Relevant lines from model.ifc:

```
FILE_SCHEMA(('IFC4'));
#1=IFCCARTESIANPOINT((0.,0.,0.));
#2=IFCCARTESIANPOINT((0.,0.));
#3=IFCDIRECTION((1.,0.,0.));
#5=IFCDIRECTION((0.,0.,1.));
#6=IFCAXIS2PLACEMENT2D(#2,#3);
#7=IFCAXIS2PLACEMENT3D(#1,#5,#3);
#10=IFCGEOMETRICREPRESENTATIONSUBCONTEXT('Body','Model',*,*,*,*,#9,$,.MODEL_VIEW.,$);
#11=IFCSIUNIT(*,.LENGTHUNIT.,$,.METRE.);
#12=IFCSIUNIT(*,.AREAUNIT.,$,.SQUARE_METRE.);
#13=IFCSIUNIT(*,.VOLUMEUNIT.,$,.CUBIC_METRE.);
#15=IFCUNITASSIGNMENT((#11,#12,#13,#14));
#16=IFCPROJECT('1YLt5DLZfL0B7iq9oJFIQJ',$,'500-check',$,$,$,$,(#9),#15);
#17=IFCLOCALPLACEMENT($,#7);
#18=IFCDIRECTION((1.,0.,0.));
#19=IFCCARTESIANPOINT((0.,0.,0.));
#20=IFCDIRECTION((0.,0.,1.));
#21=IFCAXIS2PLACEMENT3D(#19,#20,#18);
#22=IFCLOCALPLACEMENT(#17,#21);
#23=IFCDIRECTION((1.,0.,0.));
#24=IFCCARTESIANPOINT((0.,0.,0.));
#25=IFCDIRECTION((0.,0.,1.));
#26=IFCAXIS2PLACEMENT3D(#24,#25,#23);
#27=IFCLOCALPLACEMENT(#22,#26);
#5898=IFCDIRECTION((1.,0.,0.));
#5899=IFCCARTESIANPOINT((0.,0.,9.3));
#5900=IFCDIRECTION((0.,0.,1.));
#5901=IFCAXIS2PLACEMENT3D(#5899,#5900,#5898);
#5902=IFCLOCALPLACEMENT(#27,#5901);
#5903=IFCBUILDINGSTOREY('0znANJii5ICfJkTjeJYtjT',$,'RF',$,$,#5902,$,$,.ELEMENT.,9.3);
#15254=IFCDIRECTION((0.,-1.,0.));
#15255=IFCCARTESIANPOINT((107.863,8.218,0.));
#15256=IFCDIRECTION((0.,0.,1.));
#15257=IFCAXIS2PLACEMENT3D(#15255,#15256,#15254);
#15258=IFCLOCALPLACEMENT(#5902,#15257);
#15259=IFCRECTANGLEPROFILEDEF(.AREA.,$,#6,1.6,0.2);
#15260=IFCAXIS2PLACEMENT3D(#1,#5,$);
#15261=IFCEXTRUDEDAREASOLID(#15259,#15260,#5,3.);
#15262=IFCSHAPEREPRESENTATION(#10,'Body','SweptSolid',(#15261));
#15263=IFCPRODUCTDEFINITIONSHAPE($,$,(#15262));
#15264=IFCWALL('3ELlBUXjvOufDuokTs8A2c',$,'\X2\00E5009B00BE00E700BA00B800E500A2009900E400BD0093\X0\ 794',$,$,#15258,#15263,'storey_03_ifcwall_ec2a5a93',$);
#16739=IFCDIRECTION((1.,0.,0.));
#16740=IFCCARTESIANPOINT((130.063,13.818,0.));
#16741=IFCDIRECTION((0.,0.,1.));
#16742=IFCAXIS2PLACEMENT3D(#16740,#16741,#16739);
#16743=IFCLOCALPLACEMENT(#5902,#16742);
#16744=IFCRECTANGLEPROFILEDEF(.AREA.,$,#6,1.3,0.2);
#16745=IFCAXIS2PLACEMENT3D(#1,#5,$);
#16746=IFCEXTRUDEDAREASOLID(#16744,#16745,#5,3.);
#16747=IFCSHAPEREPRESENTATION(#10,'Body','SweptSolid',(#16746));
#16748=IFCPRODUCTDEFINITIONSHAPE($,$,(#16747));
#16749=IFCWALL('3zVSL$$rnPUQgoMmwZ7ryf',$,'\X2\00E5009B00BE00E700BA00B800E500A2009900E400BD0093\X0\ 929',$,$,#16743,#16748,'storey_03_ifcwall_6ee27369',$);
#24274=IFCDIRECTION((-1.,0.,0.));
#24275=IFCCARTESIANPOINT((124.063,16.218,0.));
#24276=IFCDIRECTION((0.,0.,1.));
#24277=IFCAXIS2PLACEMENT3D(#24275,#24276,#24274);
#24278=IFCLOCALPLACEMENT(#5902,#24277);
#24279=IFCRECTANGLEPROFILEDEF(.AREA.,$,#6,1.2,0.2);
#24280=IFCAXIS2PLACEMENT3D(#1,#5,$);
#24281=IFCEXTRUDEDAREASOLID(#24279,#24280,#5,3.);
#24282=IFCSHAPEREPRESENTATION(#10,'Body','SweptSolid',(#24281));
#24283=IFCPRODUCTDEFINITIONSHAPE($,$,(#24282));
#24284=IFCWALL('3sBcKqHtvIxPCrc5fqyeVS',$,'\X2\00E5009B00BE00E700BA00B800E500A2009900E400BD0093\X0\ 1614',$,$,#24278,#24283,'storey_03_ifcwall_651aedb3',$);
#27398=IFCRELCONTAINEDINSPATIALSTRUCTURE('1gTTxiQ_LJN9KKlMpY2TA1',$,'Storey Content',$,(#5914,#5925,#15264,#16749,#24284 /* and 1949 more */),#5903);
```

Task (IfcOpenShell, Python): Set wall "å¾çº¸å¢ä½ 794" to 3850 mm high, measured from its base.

```python
import ifcopenshell
import ifcopenshell.geom
import ifcopenshell.util.representation
import ifcopenshell.util.shape
import ifcopenshell.util.unit

model = ifcopenshell.open("model.ifc")
unit_scale = ifcopenshell.util.unit.calculate_unit_scale(model)
settings = ifcopenshell.geom.settings()


def volume(element):
    """Net volume in cubic metres, openings subtracted."""
    shape = ifcopenshell.geom.create_shape(settings, element)
    return ifcopenshell.util.shape.get_volume(shape.geometry)


wall = model.by_id(15264)
before = volume(wall)

body = ifcopenshell.util.representation.get_representation(wall, "Model", "Body")
solid = body.Items[0]
old_height = solid.Depth
solid.Depth = 3.85 / unit_scale
after = volume(wall)

print(f"height {old_height:g} -> {solid.Depth:g}, volume {before:.3f} -> {after:.3f} m3")

model.write("model-out.ifc")
```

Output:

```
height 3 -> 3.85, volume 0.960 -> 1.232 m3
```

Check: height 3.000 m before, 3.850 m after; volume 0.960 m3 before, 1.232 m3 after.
